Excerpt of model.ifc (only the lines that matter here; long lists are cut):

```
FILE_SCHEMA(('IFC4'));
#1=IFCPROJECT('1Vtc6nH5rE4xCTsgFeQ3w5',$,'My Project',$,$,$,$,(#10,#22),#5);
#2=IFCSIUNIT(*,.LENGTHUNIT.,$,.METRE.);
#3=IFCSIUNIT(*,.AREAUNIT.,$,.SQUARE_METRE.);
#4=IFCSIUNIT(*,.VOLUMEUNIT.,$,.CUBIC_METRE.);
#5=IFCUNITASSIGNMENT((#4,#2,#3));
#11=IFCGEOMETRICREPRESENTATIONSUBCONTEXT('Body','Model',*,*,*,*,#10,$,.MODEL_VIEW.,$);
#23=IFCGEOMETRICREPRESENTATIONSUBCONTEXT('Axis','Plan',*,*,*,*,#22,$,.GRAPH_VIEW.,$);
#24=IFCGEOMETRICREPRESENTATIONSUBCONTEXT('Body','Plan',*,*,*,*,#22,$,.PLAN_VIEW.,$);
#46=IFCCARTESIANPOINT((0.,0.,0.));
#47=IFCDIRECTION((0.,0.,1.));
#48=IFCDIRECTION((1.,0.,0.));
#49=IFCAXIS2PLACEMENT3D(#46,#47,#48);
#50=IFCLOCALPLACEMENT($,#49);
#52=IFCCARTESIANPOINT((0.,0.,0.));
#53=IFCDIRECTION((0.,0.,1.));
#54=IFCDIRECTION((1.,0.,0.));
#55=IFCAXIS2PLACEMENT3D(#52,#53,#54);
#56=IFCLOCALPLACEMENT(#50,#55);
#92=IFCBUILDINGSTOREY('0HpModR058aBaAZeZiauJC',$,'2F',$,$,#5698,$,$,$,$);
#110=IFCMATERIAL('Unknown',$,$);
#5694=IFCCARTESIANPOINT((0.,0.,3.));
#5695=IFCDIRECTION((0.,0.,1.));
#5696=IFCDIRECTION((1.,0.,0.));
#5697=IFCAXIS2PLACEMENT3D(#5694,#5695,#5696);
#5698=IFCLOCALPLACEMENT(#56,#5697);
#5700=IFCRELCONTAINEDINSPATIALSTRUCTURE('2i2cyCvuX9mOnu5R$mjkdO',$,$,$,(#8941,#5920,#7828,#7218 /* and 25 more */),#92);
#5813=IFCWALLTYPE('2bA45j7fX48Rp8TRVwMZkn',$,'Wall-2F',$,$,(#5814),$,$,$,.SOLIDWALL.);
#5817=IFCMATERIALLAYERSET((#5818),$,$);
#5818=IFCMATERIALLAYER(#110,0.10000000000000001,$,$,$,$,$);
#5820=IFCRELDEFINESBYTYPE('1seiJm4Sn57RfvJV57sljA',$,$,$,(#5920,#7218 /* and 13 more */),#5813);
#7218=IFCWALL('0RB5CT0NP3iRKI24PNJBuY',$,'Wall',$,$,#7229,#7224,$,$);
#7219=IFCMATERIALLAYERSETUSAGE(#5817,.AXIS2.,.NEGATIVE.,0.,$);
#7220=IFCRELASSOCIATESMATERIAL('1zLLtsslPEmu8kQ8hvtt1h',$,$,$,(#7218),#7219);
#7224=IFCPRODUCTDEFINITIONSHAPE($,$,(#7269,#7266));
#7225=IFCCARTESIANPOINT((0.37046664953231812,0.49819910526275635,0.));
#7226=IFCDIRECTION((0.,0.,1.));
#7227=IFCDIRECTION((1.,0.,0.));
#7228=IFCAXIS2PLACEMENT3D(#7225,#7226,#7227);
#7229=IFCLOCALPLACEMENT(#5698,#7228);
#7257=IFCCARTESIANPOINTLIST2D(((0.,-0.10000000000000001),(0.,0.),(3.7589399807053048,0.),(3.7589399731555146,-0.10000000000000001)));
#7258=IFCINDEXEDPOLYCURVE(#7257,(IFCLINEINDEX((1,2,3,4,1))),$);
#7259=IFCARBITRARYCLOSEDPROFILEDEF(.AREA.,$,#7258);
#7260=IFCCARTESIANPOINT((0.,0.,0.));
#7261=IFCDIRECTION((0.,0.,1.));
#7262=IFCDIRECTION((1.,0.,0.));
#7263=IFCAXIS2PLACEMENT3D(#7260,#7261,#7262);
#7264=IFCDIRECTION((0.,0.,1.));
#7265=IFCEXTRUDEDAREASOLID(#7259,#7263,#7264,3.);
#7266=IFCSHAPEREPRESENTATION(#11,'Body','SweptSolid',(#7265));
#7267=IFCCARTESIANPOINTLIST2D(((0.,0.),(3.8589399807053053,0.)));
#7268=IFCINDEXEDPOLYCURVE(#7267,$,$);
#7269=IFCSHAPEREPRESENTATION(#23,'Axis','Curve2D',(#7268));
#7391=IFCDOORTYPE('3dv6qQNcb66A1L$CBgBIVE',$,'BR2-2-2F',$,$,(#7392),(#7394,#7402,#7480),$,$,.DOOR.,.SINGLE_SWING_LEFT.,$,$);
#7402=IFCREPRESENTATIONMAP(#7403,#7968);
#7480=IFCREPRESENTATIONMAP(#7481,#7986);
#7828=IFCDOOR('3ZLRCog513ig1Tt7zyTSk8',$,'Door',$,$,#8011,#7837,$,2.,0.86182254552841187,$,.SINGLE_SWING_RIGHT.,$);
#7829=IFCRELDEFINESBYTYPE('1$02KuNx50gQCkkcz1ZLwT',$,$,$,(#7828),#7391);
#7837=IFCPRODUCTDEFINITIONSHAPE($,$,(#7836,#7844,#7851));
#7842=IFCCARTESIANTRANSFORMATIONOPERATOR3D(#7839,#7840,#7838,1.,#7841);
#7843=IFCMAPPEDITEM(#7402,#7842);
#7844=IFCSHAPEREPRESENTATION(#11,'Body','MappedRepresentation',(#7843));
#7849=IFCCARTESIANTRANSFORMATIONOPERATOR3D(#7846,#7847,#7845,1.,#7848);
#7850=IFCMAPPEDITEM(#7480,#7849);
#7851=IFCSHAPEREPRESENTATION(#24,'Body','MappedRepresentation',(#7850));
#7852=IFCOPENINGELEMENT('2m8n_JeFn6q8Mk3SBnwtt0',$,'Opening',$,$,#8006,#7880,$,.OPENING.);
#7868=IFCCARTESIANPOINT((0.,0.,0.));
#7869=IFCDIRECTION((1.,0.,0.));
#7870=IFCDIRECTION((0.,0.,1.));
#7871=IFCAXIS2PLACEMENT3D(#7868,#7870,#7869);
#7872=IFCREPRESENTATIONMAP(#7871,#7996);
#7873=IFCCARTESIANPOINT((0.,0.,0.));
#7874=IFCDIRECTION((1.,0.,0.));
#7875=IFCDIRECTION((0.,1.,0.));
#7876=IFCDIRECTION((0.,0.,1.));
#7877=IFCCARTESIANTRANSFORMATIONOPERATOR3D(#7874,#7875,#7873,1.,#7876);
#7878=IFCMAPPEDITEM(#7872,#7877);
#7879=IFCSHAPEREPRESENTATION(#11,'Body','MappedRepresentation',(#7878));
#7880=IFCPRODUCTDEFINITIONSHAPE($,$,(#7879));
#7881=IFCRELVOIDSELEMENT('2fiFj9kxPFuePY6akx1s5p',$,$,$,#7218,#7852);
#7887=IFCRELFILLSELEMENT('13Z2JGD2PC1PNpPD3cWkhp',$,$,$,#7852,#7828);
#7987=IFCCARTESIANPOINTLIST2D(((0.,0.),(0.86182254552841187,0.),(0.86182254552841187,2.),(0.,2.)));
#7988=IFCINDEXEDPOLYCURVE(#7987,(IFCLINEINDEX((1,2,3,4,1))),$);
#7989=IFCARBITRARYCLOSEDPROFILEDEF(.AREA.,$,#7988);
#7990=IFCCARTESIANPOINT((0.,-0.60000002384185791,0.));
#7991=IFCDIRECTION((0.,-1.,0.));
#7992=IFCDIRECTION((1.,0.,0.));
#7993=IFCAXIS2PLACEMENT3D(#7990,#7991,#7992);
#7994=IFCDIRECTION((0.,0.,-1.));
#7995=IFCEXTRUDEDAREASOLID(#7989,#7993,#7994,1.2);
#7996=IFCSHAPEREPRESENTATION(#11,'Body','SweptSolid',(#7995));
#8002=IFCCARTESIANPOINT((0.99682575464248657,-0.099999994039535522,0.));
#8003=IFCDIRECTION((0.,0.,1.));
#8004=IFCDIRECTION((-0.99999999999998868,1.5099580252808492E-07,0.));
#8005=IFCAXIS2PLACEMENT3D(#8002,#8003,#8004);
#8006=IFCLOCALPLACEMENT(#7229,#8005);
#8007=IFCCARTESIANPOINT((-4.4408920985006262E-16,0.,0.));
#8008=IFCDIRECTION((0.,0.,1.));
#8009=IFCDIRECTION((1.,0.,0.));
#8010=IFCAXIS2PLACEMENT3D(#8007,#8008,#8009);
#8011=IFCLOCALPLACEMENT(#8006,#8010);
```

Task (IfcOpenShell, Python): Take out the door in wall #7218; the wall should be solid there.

```python
import ifcopenshell
import ifcopenshell.api.feature
import ifcopenshell.api.root
import ifcopenshell.geom
import ifcopenshell.util.shape

model = ifcopenshell.open("model.ifc")
settings = ifcopenshell.geom.settings()


def volume(element):
    """Net volume in cubic metres, openings subtracted."""
    shape = ifcopenshell.geom.create_shape(settings, element)
    return ifcopenshell.util.shape.get_volume(shape.geometry)


door = model.by_id(7828)
opening = door.FillsVoids[0].RelatingOpeningElement
wall = opening.VoidsElements[0].RelatingBuildingElement
before = volume(wall)

ifcopenshell.api.root.remove_product(model, product=door)
ifcopenshell.api.feature.remove_feature(model, feature=opening)

after = volume(wall)

print(f"wall volume {before:.3f} -> {after:.3f} m3")

model.write("model_v2.ifc")
```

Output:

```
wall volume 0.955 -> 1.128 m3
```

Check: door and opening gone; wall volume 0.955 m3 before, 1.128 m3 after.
